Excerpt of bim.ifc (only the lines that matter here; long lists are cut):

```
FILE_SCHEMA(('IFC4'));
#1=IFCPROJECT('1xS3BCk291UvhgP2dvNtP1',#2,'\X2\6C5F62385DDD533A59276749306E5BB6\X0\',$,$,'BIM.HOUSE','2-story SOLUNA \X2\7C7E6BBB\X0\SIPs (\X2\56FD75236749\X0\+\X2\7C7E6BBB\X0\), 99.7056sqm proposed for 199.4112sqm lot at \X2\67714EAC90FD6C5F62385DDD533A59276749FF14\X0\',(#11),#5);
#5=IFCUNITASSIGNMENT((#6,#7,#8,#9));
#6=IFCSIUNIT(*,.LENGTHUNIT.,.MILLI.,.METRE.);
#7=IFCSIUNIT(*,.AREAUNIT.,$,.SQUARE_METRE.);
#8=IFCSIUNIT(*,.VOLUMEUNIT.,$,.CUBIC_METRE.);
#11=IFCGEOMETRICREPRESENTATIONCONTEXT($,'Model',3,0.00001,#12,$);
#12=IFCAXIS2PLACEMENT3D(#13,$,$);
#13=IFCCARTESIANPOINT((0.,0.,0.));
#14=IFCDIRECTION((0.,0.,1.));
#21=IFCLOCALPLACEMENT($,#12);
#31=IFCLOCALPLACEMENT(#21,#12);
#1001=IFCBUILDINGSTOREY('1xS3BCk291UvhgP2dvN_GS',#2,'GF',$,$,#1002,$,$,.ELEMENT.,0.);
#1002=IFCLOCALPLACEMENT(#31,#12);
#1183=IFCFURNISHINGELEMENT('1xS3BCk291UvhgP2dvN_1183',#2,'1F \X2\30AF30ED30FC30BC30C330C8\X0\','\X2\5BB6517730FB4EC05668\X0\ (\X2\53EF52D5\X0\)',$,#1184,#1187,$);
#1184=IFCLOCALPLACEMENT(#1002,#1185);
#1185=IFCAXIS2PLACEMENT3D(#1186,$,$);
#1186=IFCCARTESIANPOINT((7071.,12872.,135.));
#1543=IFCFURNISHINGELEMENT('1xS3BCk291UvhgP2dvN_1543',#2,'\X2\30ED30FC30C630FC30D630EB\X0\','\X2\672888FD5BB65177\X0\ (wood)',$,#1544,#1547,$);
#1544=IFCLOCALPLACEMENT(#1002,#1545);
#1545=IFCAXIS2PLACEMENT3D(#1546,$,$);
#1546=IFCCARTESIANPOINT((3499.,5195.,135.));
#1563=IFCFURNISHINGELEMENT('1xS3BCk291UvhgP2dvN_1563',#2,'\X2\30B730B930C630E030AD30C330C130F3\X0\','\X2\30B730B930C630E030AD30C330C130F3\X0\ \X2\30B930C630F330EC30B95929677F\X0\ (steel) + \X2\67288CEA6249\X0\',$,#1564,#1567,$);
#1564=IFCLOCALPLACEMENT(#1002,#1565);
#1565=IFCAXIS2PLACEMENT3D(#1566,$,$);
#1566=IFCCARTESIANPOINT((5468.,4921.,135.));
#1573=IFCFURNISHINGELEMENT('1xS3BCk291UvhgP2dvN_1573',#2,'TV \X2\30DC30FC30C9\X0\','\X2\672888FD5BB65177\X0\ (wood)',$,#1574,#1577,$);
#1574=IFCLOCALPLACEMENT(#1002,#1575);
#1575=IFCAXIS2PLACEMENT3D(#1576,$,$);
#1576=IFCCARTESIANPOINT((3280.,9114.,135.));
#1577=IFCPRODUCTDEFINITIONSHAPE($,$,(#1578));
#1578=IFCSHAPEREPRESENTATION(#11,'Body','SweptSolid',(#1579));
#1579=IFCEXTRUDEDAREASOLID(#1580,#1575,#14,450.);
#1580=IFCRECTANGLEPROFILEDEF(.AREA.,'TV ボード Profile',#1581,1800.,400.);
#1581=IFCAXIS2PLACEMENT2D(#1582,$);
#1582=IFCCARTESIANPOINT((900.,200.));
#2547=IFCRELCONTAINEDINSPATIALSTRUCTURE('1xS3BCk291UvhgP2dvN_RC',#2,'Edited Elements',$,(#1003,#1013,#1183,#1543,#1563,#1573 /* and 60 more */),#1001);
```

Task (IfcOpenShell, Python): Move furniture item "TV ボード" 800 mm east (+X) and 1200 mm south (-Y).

```python
import ifcopenshell
import ifcopenshell.api.geometry
import ifcopenshell.util.placement
import ifcopenshell.util.unit

model = ifcopenshell.open("bim.ifc")
unit_scale = ifcopenshell.util.unit.calculate_unit_scale(model)

item = model.by_guid("1xS3BCk291UvhgP2dvN_1573")
matrix = ifcopenshell.util.placement.get_local_placement(item.ObjectPlacement)
matrix[0, 3] += 0.8 / unit_scale
matrix[1, 3] -= 1.2 / unit_scale
ifcopenshell.api.geometry.edit_object_placement(model, product=item, matrix=matrix, is_si=False)

print(ifcopenshell.util.placement.get_local_placement(item.ObjectPlacement).round(3) + 0.0)

model.write("bim_rev.ifc")
```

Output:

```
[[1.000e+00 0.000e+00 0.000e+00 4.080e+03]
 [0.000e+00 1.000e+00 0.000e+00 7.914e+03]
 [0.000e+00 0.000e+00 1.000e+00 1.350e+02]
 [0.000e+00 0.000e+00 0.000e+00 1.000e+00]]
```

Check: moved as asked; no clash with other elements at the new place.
